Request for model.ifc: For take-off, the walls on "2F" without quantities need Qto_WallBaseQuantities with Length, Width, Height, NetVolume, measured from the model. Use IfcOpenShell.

First a look at what the model holds.

```python
import ifcopenshell
import ifcopenshell.util.element
import ifcopenshell.util.unit

model = ifcopenshell.open("model.ifc")
print(model.schema)
for unit_type in ("LENGTHUNIT", "AREAUNIT", "VOLUMEUNIT"):
    print(unit_type, ifcopenshell.util.unit.calculate_unit_scale(model, unit_type))
storey = next(s for s in model.by_type("IfcBuildingStorey") if s.Name == "2F")
walls = [e for e in ifcopenshell.util.element.get_decomposition(storey) if e.is_a("IfcWall")]
for e in sorted(walls, key=lambda e: e.id()):
    print(e.id(), e.is_a(), e.Name, list(ifcopenshell.util.element.get_psets(e, qtos_only=True)), sep=" | ")
```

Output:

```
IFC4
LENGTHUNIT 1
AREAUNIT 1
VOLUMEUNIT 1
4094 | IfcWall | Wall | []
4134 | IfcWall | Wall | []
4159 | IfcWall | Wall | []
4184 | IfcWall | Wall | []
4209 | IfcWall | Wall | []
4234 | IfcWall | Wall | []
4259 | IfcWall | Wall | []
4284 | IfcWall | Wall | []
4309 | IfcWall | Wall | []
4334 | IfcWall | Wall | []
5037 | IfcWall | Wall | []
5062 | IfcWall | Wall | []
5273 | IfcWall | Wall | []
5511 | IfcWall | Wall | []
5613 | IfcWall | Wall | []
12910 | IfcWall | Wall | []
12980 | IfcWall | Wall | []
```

```python
import ifcopenshell
import ifcopenshell.api.pset
import ifcopenshell.geom
import ifcopenshell.util.element
import ifcopenshell.util.shape
import ifcopenshell.util.unit

model = ifcopenshell.open("model.ifc")
unit_scale = ifcopenshell.util.unit.calculate_unit_scale(model)
volume_scale = ifcopenshell.util.unit.calculate_unit_scale(model, "VOLUMEUNIT")
settings = ifcopenshell.geom.settings()

storey = next(s for s in model.by_type("IfcBuildingStorey") if s.Name == "2F")
walls = [e for e in ifcopenshell.util.element.get_decomposition(storey) if e.is_a("IfcWall")]

for e in sorted(walls, key=lambda e: e.id()):
    if ifcopenshell.util.element.get_psets(e, qtos_only=True, should_inherit=False):
        continue
    # Geometry comes back in metres, in the element's own axes.
    shape = ifcopenshell.geom.create_shape(settings, e)
    values = {
        "Length": ifcopenshell.util.shape.get_x(shape.geometry) / unit_scale,
        "Width": ifcopenshell.util.shape.get_y(shape.geometry) / unit_scale,
        "Height": ifcopenshell.util.shape.get_z(shape.geometry) / unit_scale,
        "NetVolume": ifcopenshell.util.shape.get_volume(shape.geometry) / volume_scale,
    }
    qto = ifcopenshell.api.pset.add_qto(model, product=e, name="Qto_WallBaseQuantities")
    ifcopenshell.api.pset.edit_qto(model, qto=qto, properties=values)
    print(e.id(), {k: round(v, 3) for k, v in values.items()})

model.write("model_edited.ifc")
```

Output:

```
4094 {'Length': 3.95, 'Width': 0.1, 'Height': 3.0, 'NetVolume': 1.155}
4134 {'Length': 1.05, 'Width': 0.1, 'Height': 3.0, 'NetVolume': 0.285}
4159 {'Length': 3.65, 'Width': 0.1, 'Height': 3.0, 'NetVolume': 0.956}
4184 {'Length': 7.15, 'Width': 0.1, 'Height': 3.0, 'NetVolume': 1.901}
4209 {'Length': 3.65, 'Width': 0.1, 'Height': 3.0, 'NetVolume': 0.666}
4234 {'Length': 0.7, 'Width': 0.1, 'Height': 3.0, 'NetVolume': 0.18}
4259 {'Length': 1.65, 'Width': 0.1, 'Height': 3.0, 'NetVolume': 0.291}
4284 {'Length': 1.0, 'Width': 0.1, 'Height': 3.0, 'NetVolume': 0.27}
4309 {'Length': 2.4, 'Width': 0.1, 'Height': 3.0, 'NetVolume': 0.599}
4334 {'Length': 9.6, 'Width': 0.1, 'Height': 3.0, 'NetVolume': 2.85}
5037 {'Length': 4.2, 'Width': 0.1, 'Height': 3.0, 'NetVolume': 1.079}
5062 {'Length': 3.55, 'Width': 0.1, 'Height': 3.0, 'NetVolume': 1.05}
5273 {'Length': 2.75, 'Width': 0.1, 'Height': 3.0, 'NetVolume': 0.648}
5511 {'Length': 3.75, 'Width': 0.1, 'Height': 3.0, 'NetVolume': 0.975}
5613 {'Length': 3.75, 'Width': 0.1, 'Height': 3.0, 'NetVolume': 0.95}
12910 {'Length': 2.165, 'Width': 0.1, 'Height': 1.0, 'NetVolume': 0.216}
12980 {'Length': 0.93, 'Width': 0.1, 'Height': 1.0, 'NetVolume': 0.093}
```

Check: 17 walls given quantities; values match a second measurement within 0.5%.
